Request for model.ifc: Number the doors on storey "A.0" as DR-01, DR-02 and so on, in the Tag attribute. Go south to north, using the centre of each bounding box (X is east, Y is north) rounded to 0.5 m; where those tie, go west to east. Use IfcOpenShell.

First a look at what the model holds.

```python
import ifcopenshell
import ifcopenshell.util.element
import ifcopenshell.util.placement

model = ifcopenshell.open("model.ifc")
print(model.schema)
storey = next(s for s in model.by_type("IfcBuildingStorey") if s.Name == "A.0")
doors = [e for e in ifcopenshell.util.element.get_decomposition(storey) if e.is_a("IfcDoor")]
for e in sorted(doors, key=lambda e: e.id()):
    origin = ifcopenshell.util.placement.get_local_placement(e.ObjectPlacement)[:3, 3]
    print(e.id(), e.Tag, e.Name, origin.round(2) + 0.0, sep=" | ")
```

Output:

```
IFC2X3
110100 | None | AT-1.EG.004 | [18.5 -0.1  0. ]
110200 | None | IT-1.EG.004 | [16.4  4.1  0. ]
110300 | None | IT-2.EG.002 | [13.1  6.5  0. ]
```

```python
import ifcopenshell
import ifcopenshell.geom
import ifcopenshell.util.element
import ifcopenshell.util.shape

model = ifcopenshell.open("model.ifc")
settings = ifcopenshell.geom.settings()
settings.set("use-world-coords", True)


def centre(element):
    shape = ifcopenshell.geom.create_shape(settings, element)
    return ifcopenshell.util.shape.get_bbox_centroid(shape.geometry)


storey = next(s for s in model.by_type("IfcBuildingStorey") if s.Name == "A.0")
doors = [e for e in ifcopenshell.util.element.get_decomposition(storey) if e.is_a("IfcDoor")]

# Insertion points can sit at a corner or the storey origin, so sort by the geometry (in metres).
centres = {e: centre(e) for e in doors}
doors.sort(key=lambda e: (round(centres[e][1] / 0.5), centres[e][0]))

for i, e in enumerate(doors, start=1):
    number = f"DR-{i:02d}"
    e.Tag = number
    print(e.id(), number)

model.write("model_edited.ifc")
```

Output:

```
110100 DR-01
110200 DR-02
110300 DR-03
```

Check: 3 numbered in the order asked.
